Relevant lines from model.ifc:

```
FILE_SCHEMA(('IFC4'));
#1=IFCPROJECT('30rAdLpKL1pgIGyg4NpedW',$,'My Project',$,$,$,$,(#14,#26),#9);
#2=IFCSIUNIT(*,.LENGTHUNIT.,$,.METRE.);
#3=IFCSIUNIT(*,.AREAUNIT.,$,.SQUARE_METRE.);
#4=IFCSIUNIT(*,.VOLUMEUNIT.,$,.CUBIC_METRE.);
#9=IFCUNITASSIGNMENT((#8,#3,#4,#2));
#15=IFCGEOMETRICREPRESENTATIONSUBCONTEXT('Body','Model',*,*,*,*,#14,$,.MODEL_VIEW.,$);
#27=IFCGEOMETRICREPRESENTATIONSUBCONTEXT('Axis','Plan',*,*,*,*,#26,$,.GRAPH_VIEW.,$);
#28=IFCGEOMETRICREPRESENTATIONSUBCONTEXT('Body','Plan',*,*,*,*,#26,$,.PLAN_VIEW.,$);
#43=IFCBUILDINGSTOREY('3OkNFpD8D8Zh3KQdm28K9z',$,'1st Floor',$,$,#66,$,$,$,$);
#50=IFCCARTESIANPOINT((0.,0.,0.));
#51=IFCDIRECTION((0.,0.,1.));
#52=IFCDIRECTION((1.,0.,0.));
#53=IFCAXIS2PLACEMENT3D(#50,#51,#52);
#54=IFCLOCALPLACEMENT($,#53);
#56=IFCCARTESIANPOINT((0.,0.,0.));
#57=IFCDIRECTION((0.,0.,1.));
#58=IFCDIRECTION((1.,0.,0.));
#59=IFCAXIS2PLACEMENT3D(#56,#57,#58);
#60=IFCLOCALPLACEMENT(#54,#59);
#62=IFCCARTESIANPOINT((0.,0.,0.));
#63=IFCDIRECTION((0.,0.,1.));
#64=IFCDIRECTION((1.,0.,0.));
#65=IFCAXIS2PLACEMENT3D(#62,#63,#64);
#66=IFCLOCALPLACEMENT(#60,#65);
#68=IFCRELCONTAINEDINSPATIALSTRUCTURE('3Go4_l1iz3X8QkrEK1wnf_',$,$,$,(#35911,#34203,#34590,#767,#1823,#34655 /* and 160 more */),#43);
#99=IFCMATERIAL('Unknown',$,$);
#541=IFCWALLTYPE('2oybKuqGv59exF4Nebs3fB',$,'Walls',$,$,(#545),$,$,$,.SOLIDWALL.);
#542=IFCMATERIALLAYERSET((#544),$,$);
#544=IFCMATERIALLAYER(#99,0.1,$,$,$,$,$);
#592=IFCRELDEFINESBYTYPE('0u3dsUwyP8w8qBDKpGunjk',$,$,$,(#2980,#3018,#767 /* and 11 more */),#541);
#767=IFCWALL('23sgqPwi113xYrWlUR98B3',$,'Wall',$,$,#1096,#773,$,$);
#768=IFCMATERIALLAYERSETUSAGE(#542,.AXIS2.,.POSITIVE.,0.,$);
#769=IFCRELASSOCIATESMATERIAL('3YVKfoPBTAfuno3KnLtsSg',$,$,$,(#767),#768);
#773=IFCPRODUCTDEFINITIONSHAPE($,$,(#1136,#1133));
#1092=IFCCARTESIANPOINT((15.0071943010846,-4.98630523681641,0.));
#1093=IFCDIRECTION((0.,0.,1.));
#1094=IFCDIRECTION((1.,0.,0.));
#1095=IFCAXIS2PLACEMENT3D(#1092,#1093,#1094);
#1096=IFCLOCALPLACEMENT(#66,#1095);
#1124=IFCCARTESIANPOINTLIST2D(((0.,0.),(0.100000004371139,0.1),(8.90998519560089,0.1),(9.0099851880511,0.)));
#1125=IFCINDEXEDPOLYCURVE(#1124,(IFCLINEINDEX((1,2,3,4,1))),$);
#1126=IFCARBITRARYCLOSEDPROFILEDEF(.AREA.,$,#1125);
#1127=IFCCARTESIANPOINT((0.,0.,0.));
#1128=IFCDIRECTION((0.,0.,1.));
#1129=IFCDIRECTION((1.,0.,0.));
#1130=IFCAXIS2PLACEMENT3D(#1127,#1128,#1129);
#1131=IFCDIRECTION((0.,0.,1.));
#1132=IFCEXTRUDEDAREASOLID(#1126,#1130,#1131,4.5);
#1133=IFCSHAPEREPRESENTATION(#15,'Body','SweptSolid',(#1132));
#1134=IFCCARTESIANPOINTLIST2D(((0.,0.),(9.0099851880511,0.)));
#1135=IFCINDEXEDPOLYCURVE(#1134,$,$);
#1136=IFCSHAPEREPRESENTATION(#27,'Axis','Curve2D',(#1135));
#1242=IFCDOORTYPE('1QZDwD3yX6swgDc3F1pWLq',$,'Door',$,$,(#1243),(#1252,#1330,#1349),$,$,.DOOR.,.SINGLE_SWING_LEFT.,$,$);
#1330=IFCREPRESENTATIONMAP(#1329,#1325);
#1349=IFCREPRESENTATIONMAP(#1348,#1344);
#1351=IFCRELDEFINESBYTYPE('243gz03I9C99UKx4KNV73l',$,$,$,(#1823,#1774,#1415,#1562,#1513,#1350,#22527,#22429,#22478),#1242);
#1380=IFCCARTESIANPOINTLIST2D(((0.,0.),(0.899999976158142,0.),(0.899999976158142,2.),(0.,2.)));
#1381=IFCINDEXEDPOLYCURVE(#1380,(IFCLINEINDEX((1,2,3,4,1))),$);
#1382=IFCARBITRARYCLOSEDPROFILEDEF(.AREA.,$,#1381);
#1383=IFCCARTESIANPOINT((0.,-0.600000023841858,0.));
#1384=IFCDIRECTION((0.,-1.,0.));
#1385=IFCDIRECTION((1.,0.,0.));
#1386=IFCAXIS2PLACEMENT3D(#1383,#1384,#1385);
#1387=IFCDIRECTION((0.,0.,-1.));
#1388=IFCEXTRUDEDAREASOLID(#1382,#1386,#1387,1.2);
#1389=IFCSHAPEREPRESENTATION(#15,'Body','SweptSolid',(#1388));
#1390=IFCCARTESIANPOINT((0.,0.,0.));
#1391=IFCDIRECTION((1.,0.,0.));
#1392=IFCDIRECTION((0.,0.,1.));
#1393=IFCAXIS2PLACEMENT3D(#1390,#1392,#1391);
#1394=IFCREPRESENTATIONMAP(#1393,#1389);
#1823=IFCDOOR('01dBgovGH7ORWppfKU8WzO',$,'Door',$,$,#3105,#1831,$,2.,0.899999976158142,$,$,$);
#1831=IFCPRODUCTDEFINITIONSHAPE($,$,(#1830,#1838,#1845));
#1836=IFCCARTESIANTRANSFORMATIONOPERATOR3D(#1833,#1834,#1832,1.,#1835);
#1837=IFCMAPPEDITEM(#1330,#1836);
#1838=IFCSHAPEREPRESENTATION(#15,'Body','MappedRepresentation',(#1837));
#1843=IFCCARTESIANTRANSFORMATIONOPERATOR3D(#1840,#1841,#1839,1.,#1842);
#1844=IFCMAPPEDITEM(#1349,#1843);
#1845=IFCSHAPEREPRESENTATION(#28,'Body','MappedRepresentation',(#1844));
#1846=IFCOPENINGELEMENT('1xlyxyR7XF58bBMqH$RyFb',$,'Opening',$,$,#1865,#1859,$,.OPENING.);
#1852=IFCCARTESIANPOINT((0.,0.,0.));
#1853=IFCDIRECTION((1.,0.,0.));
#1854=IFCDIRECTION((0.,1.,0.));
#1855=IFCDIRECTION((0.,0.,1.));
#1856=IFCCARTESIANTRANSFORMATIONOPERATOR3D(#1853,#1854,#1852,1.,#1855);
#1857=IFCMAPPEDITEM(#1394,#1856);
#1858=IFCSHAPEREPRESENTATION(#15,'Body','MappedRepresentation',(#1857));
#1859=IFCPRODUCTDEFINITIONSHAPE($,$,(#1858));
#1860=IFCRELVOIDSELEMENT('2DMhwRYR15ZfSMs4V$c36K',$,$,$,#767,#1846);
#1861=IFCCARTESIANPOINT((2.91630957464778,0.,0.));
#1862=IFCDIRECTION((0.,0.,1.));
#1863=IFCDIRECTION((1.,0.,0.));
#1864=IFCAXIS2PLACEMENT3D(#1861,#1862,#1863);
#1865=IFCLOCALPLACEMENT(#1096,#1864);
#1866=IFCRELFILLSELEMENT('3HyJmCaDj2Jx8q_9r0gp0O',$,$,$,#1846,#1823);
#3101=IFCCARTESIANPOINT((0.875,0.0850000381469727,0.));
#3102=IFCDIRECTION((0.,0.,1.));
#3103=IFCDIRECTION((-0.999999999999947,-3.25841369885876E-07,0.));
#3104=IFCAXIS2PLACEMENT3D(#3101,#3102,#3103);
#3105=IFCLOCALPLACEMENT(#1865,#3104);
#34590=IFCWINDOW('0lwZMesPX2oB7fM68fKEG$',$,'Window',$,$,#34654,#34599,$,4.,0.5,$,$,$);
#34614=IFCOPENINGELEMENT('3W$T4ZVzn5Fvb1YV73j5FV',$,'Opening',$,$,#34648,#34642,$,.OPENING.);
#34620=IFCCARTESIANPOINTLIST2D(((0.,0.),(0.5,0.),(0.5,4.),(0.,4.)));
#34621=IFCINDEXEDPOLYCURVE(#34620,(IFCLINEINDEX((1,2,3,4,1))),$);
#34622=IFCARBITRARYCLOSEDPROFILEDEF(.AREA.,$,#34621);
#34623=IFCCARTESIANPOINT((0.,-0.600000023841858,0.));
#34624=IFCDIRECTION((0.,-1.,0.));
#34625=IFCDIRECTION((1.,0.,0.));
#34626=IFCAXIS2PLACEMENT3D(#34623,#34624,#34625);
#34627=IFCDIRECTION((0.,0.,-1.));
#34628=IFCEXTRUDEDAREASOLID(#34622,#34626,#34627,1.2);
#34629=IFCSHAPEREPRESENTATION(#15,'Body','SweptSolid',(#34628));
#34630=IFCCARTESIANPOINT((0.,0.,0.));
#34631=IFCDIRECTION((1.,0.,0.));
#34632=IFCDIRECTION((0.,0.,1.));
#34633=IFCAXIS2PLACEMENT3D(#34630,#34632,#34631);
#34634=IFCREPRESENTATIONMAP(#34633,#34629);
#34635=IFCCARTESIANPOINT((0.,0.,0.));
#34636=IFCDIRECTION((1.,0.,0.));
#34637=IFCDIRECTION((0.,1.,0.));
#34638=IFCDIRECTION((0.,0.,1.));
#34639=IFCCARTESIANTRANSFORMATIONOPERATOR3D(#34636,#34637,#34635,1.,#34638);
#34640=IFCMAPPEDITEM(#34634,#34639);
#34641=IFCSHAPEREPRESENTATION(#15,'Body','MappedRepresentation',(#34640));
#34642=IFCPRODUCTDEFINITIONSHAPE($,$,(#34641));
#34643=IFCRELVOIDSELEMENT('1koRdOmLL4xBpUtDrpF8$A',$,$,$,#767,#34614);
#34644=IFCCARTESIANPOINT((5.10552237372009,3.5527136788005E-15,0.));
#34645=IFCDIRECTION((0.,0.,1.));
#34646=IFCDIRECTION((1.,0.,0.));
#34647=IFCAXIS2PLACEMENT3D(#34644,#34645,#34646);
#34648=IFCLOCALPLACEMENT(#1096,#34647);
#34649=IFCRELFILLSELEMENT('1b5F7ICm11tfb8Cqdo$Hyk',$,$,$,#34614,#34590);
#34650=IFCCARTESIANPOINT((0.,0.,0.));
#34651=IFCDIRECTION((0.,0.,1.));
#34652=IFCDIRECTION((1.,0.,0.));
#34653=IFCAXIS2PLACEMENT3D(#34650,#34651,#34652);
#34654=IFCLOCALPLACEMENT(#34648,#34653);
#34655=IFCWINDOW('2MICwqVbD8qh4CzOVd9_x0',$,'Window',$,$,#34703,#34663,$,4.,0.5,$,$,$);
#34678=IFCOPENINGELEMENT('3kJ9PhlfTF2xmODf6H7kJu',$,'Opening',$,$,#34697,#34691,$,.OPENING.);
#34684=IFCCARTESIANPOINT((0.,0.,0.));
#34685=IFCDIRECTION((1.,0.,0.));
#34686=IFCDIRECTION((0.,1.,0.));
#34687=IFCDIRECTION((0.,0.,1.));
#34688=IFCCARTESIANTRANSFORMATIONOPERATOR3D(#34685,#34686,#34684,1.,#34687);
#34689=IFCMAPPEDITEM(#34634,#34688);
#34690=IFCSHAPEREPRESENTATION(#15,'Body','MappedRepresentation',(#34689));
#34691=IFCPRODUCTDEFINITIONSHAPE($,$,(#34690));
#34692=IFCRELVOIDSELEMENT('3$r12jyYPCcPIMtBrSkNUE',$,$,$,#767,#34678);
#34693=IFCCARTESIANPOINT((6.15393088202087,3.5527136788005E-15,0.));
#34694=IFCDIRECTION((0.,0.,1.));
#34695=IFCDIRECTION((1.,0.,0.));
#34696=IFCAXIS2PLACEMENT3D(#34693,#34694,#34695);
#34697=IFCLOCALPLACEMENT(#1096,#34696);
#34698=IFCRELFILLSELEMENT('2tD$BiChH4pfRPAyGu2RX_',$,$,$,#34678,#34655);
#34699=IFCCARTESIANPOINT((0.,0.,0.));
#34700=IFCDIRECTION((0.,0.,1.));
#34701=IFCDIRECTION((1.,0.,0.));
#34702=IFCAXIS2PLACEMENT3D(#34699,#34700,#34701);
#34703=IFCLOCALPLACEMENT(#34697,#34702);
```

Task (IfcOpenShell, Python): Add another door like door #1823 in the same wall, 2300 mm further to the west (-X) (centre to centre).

```python
import ifcopenshell
import ifcopenshell.api.feature
import ifcopenshell.api.geometry
import ifcopenshell.api.root
import ifcopenshell.geom
import ifcopenshell.util.element
import ifcopenshell.util.placement
import ifcopenshell.util.shape

model = ifcopenshell.open("model.ifc")
settings = ifcopenshell.geom.settings()


def volume(element):
    """Net volume in cubic metres, openings subtracted."""
    shape = ifcopenshell.geom.create_shape(settings, element)
    return ifcopenshell.util.shape.get_volume(shape.geometry)


door = model.by_id(1823)
opening = door.FillsVoids[0].RelatingOpeningElement
wall = opening.VoidsElements[0].RelatingBuildingElement
before = volume(wall)
shift = ifcopenshell.util.placement.get_local_placement(wall.ObjectPlacement)[:3, 0] * -2.3

# copy_class copies the void relationship, type, container and properties, but no geometry.
new_opening = ifcopenshell.api.root.copy_class(model, product=opening)
new_opening.Representation = ifcopenshell.util.element.copy_deep(
    model, opening.Representation, exclude=["IfcGeometricRepresentationContext", "IfcRepresentationMap"]
)
new_door = ifcopenshell.api.root.copy_class(model, product=door)
new_door.Representation = ifcopenshell.util.element.copy_deep(
    model, door.Representation, exclude=["IfcGeometricRepresentationContext", "IfcRepresentationMap"]
)
ifcopenshell.api.feature.add_filling(model, opening=new_opening, element=new_door)

for old, new in ((opening, new_opening), (door, new_door)):
    matrix = ifcopenshell.util.placement.get_local_placement(old.ObjectPlacement)
    matrix[:3, 3] += shift
    ifcopenshell.api.geometry.edit_object_placement(model, product=new, matrix=matrix, is_si=False)

after = volume(wall)

print(f"wall volume {before:.3f} -> {after:.3f} m3")

model.write("model_v2.ifc")
```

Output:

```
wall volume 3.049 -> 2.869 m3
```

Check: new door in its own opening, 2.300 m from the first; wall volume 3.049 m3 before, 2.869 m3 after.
